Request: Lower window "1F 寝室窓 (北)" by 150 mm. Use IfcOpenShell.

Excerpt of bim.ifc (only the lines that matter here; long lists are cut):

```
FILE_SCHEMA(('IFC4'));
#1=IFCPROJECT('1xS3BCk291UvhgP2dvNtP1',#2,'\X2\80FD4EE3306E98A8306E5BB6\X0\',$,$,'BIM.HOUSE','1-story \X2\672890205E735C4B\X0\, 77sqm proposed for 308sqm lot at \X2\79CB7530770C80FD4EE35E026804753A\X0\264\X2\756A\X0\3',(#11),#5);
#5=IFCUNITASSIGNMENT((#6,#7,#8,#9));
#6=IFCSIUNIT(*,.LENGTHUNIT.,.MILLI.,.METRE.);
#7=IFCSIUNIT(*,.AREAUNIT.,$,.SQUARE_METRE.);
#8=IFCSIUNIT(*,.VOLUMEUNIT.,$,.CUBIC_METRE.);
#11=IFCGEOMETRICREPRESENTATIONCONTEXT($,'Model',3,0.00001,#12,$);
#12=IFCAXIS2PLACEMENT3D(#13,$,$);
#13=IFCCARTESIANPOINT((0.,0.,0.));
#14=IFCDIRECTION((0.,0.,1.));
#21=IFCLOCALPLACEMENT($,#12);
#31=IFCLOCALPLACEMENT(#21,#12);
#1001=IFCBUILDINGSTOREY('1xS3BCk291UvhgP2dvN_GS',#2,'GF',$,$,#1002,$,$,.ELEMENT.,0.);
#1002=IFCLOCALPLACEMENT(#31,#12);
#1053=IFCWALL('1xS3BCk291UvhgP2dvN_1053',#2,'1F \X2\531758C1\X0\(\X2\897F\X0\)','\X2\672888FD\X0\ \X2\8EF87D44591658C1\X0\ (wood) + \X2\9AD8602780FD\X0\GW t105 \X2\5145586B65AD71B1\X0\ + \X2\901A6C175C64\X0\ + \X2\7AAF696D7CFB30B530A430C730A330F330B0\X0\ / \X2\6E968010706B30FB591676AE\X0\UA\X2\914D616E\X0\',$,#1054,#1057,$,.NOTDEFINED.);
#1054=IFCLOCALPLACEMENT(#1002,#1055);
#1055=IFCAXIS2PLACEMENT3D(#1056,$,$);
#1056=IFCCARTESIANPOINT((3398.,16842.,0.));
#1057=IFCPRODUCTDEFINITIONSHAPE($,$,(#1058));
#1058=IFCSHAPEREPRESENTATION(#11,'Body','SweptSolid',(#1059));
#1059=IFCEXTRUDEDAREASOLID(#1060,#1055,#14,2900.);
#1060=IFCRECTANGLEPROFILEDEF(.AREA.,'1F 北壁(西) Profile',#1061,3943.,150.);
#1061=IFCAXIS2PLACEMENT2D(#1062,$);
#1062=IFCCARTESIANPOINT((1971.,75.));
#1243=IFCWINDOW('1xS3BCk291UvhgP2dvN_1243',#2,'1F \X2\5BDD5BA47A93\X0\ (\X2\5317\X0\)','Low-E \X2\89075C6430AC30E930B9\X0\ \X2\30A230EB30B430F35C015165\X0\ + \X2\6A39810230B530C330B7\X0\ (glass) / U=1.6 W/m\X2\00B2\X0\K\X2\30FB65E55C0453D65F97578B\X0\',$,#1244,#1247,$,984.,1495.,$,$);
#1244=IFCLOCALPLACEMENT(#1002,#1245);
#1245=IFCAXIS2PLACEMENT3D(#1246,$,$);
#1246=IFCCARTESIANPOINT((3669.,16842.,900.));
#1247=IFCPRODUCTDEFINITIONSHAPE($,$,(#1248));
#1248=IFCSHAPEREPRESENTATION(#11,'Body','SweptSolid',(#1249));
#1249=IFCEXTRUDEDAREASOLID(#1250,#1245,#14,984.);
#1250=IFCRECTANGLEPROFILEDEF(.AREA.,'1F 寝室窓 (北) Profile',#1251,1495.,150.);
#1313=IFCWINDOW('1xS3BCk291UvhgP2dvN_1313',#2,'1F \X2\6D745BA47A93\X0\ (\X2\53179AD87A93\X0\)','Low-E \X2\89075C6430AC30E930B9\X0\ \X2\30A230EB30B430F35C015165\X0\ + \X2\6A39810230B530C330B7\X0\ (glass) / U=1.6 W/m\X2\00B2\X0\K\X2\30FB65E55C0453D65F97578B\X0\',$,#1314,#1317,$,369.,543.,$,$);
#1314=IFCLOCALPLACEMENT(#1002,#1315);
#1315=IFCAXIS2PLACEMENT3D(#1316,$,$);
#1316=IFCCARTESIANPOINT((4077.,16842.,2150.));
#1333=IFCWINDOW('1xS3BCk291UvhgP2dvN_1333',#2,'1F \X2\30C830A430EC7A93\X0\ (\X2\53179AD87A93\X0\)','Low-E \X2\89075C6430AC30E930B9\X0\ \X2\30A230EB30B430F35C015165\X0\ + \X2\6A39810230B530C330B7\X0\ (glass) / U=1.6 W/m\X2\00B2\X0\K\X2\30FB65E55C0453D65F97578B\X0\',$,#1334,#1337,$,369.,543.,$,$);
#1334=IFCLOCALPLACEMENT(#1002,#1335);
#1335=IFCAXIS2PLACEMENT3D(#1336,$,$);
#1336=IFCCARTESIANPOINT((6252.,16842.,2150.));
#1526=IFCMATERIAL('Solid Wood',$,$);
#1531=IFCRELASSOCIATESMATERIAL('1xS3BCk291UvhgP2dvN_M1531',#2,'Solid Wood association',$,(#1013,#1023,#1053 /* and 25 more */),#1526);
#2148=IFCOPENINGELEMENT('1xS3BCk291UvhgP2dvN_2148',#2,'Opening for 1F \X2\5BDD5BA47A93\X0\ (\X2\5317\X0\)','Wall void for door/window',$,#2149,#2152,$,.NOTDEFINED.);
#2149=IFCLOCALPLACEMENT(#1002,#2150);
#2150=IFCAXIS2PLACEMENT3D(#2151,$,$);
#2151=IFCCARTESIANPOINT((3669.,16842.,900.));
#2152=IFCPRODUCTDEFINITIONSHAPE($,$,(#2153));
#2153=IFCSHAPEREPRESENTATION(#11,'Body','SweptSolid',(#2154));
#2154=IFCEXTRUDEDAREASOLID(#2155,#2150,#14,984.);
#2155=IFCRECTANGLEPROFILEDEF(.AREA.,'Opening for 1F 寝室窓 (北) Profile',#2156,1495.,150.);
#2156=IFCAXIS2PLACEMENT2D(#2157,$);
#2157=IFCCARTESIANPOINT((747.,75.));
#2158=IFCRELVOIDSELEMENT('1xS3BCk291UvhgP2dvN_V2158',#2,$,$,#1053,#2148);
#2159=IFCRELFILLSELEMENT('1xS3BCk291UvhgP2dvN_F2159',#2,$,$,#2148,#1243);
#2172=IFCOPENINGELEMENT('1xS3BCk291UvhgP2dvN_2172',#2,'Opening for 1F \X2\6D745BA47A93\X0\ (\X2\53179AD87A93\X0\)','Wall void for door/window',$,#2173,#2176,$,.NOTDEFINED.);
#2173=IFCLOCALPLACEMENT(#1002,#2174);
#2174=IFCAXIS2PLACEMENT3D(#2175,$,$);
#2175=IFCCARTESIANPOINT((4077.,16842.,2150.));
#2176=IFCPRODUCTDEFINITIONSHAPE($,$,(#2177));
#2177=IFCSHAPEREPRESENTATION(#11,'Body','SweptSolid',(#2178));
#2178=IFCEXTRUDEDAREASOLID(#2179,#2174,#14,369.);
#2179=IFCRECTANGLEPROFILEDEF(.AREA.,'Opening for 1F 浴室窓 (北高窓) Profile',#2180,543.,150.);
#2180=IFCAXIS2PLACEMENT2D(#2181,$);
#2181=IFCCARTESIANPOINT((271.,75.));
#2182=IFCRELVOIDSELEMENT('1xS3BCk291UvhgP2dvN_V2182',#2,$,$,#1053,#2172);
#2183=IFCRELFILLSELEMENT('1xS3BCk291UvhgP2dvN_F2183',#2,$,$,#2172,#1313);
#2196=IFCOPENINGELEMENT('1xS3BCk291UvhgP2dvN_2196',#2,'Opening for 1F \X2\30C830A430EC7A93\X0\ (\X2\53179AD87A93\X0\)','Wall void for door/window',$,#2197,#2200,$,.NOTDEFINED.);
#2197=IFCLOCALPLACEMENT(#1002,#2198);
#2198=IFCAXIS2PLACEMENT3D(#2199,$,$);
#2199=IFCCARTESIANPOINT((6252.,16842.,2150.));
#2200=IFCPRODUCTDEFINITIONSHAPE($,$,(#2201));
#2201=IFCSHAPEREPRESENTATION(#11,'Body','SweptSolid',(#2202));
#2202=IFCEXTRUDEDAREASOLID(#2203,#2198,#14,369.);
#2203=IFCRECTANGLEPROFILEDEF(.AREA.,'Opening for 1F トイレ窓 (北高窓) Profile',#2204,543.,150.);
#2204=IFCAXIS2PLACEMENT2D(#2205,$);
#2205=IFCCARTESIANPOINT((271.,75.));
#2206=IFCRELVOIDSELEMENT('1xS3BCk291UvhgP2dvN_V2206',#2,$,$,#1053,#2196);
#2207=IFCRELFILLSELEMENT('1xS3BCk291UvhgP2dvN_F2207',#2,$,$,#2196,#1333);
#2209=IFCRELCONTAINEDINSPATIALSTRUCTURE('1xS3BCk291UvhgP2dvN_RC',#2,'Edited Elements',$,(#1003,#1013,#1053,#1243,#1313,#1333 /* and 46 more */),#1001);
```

```python
import numpy as np
import ifcopenshell
import ifcopenshell.api.geometry
import ifcopenshell.util.placement
import ifcopenshell.util.unit

model = ifcopenshell.open("bim.ifc")
unit_scale = ifcopenshell.util.unit.calculate_unit_scale(model)

window = model.by_guid("1xS3BCk291UvhgP2dvN_1243")
opening = window.FillsVoids[0].RelatingOpeningElement
dz = -0.15 / unit_scale

shift = np.array([0.0, 0.0, dz])
# The window is not placed relative to its opening, so move both.
for product in (opening, window):
    matrix = ifcopenshell.util.placement.get_local_placement(product.ObjectPlacement)
    matrix[:3, 3] += shift
    ifcopenshell.api.geometry.edit_object_placement(model, product=product, matrix=matrix, is_si=False)

print(f"moved by {dz * unit_scale:+.3f} m")

model.write("bim-out.ifc")
```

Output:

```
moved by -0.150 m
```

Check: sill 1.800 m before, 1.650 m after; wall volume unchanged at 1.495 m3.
